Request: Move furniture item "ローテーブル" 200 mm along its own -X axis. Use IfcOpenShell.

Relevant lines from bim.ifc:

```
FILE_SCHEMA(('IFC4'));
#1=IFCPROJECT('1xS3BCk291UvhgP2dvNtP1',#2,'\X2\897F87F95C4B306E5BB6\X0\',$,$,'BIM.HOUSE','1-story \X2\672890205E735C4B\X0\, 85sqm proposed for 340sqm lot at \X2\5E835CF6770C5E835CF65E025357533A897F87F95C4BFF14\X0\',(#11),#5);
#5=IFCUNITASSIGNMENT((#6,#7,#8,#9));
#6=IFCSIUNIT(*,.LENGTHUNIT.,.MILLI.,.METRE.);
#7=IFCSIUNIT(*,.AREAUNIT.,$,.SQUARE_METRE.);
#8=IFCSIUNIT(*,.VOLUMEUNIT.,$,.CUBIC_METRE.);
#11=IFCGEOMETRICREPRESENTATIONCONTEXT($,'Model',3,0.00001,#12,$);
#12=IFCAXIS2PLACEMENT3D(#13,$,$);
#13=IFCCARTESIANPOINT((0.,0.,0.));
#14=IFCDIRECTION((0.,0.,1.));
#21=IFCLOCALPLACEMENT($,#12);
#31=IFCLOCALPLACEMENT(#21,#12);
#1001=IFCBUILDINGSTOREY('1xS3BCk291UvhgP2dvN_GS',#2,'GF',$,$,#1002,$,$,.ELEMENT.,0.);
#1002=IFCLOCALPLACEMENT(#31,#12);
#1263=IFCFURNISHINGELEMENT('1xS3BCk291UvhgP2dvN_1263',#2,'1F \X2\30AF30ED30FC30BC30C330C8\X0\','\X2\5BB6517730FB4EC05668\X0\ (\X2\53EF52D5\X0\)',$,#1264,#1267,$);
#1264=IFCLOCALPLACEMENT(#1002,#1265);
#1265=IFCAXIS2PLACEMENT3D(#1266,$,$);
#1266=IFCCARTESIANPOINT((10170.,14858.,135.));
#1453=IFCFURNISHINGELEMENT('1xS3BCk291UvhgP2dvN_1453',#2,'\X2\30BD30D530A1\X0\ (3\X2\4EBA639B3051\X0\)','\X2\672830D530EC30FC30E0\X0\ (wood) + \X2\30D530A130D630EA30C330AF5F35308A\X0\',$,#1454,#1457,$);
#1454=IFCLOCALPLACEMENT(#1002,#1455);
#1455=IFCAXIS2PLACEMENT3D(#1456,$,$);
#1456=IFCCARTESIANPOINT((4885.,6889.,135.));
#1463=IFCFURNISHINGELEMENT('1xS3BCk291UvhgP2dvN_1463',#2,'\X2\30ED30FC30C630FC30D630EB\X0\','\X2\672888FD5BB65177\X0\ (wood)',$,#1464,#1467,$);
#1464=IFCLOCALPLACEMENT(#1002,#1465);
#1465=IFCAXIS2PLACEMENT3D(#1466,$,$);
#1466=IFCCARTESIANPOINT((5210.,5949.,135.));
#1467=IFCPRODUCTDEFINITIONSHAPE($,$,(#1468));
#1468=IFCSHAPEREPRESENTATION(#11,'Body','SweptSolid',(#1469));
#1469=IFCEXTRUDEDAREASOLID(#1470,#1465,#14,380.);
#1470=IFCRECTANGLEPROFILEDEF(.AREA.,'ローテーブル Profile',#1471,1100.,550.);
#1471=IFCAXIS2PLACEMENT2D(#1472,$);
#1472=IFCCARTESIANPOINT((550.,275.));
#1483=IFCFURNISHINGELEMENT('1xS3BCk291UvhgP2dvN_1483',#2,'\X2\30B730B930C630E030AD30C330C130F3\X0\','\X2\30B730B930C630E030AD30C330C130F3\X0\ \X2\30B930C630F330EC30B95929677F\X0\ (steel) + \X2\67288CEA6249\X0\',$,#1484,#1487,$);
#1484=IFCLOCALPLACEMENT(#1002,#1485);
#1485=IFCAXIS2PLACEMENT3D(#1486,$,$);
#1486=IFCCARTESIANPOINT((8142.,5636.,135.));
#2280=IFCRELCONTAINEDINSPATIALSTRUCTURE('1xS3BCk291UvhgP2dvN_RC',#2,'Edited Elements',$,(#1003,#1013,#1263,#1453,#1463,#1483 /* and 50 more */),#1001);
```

```python
import ifcopenshell
import ifcopenshell.api.geometry
import ifcopenshell.util.placement

model = ifcopenshell.open("bim.ifc")

item = model.by_id(1463)
matrix = ifcopenshell.util.placement.get_local_placement(item.ObjectPlacement)
matrix[:3, 3] -= matrix[:3, 0] * 200.0
ifcopenshell.api.geometry.edit_object_placement(model, product=item, matrix=matrix, is_si=False)

print(ifcopenshell.util.placement.get_local_placement(item.ObjectPlacement).round(3) + 0.0)

model.write("bim_v2.ifc")
```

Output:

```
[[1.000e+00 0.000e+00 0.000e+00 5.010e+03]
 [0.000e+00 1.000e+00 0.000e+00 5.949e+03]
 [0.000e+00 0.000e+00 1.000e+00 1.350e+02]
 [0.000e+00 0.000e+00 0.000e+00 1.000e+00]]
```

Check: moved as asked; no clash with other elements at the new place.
